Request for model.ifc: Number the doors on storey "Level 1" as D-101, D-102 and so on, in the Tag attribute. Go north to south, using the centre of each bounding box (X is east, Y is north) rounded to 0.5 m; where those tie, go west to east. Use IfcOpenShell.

First a look at what the model holds.

```python
import ifcopenshell
import ifcopenshell.util.element
import ifcopenshell.util.placement

model = ifcopenshell.open("model.ifc")
print(model.schema)
storey = next(s for s in model.by_type("IfcBuildingStorey") if s.Name == "Level 1")
doors = [e for e in ifcopenshell.util.element.get_decomposition(storey) if e.is_a("IfcDoor")]
for e in sorted(doors, key=lambda e: e.id()):
    origin = ifcopenshell.util.placement.get_local_placement(e.ObjectPlacement)[:3, 3]
    print(e.id(), e.Tag, e.Name, origin.round(2) + 0.0, sep=" | ")
```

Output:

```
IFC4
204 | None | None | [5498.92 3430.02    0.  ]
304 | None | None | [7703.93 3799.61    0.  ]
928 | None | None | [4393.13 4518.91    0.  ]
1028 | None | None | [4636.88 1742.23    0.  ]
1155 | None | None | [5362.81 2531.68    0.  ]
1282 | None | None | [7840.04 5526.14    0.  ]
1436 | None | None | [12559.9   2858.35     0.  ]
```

```python
import ifcopenshell
import ifcopenshell.geom
import ifcopenshell.util.element
import ifcopenshell.util.shape

model = ifcopenshell.open("model.ifc")
settings = ifcopenshell.geom.settings()
settings.set("use-world-coords", True)


def centre(element):
    shape = ifcopenshell.geom.create_shape(settings, element)
    return ifcopenshell.util.shape.get_bbox_centroid(shape.geometry)


storey = next(s for s in model.by_type("IfcBuildingStorey") if s.Name == "Level 1")
doors = [e for e in ifcopenshell.util.element.get_decomposition(storey) if e.is_a("IfcDoor")]

# Insertion points can sit at a corner or the storey origin, so sort by the geometry (in metres).
centres = {e: centre(e) for e in doors}
doors.sort(key=lambda e: (-round(centres[e][1] / 0.5), centres[e][0]))

for i, e in enumerate(doors, start=1):
    number = f"D-1{i:02d}"
    e.Tag = number
    print(e.id(), number)

model.write("model_updated.ifc")
```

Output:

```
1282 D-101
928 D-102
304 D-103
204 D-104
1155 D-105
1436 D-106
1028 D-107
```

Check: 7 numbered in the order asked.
